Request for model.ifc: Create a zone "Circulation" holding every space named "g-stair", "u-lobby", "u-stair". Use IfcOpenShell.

First a look at what the model holds.

```python
import ifcopenshell

model = ifcopenshell.open("model.ifc")
print(model.schema)
seen = {}
for space in model.by_type("IfcSpace"):
    seen[space.LongName] = seen.get(space.LongName, 0) + 1
for name, count in sorted(seen.items(), key=str):
    print(count, "x", name)
print("zones:", [z.Name for z in model.by_type("IfcZone")][:20])
```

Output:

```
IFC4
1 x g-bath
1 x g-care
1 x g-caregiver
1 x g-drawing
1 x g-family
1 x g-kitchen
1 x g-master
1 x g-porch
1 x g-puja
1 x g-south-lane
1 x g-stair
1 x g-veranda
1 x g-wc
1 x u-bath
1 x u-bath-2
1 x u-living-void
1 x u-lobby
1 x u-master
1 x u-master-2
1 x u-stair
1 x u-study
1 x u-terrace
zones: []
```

```python
import ifcopenshell
import ifcopenshell.api.group
import ifcopenshell.api.root

model = ifcopenshell.open("model.ifc")

names = {"g-stair", "u-lobby", "u-stair"}
spaces = [s for s in model.by_type("IfcSpace") if s.LongName in names]

zone = ifcopenshell.api.root.create_entity(model, ifc_class="IfcZone", name="Circulation")
ifcopenshell.api.group.assign_group(model, products=spaces, group=zone)
print(len(spaces), "spaces in", zone.Name)

model.write("model_rev.ifc")
```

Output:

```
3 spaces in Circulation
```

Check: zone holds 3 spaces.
